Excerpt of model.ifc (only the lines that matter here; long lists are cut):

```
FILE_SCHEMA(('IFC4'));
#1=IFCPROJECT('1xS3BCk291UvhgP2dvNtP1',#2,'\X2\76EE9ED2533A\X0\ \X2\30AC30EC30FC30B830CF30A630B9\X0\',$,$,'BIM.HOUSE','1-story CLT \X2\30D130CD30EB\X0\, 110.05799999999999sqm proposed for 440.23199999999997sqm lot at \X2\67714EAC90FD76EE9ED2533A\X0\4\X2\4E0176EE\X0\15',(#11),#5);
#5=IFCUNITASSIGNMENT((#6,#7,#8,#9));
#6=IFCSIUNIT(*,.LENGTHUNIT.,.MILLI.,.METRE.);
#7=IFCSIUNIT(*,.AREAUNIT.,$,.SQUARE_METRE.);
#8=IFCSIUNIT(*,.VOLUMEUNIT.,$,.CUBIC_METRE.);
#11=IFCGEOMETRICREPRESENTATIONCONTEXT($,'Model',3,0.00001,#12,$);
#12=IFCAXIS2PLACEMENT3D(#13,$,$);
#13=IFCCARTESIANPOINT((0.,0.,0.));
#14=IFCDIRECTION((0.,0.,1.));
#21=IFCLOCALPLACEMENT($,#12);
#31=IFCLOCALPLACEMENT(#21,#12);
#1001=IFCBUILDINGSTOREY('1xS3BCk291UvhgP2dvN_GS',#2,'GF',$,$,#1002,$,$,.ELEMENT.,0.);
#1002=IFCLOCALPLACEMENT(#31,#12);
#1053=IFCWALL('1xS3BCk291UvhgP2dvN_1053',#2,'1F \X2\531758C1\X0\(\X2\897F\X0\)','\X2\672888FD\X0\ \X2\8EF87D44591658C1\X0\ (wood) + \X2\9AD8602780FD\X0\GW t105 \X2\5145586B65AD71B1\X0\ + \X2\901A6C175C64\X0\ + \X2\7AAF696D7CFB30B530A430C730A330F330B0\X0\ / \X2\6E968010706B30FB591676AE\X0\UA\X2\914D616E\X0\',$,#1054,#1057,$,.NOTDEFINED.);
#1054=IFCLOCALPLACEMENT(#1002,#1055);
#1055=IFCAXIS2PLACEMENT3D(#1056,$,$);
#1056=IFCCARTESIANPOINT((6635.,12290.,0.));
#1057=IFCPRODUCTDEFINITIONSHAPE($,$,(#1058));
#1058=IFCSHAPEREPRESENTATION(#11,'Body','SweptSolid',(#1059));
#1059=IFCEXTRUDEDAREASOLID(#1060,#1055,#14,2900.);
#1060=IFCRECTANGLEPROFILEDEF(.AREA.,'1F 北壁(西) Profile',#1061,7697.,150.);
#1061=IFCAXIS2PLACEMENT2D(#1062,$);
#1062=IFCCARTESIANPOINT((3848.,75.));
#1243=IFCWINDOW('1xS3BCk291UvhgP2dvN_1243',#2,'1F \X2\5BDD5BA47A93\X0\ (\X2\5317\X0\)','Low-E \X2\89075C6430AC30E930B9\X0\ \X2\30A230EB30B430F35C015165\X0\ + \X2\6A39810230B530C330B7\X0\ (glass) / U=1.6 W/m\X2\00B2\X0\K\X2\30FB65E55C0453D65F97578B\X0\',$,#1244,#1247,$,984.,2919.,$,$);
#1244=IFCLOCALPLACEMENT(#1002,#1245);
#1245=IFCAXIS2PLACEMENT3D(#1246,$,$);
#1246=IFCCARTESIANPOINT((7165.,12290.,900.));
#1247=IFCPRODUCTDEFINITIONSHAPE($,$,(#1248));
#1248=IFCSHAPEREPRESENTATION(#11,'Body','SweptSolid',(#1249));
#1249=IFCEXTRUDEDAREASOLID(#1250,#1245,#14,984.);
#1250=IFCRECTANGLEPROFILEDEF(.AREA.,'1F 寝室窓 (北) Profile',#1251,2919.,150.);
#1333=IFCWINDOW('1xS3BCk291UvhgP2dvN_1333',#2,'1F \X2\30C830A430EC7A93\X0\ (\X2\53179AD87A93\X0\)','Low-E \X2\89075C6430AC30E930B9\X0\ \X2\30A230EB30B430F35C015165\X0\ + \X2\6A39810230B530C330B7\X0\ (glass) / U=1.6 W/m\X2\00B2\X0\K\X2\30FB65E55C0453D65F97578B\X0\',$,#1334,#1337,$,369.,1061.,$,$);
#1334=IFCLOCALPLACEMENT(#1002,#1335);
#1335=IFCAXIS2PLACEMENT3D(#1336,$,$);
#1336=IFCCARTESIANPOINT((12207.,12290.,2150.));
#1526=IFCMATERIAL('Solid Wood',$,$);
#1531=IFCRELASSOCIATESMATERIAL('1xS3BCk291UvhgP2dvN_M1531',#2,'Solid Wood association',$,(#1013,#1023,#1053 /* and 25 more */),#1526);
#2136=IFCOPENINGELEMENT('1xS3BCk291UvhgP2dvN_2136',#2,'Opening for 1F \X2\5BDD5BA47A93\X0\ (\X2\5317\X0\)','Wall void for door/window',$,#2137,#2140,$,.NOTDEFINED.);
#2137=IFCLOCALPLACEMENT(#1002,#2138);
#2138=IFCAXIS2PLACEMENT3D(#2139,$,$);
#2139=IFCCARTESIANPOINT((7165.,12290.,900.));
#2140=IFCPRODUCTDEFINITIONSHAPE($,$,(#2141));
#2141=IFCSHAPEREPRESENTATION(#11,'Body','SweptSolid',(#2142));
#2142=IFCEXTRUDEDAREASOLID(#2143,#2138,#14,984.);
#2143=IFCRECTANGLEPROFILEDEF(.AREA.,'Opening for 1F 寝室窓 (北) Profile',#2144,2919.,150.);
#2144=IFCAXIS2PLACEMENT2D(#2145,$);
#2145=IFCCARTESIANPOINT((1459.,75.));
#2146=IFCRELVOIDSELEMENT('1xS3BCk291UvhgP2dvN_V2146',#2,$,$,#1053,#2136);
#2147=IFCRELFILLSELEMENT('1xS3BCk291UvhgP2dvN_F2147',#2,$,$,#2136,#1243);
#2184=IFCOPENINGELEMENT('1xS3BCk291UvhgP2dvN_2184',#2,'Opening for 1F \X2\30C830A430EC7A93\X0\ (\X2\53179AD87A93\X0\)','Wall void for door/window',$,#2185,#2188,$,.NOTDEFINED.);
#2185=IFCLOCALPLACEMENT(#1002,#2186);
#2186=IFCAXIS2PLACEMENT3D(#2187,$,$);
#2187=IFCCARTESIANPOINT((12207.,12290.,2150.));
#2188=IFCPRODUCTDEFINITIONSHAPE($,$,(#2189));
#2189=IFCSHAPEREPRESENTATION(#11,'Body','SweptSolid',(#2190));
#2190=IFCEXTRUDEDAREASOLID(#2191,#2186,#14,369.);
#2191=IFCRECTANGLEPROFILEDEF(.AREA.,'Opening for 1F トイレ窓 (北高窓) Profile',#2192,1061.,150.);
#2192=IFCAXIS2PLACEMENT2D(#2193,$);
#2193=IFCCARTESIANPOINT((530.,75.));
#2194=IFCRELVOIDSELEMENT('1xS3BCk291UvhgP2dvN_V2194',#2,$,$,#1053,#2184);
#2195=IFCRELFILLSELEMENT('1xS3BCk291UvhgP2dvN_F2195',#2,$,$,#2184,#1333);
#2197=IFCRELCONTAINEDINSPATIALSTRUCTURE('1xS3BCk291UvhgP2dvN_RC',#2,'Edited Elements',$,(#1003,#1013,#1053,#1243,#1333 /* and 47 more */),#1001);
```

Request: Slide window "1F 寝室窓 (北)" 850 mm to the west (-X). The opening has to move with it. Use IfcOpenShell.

```python
import ifcopenshell
import ifcopenshell.api.geometry
import ifcopenshell.util.placement
import ifcopenshell.util.unit

model = ifcopenshell.open("model.ifc")
unit_scale = ifcopenshell.util.unit.calculate_unit_scale(model)

window = model.by_guid("1xS3BCk291UvhgP2dvN_1243")
opening = window.FillsVoids[0].RelatingOpeningElement
wall = opening.VoidsElements[0].RelatingBuildingElement

wall_matrix = ifcopenshell.util.placement.get_local_placement(wall.ObjectPlacement)
shift = wall_matrix[:3, 0] * -0.85 / unit_scale
before = ifcopenshell.util.placement.get_local_placement(window.ObjectPlacement)[:3, 3].copy()

# The window is not placed relative to its opening, so move both.
for product in (opening, window):
    matrix = ifcopenshell.util.placement.get_local_placement(product.ObjectPlacement)
    matrix[:3, 3] += shift
    ifcopenshell.api.geometry.edit_object_placement(model, product=product, matrix=matrix, is_si=False)

after = ifcopenshell.util.placement.get_local_placement(window.ObjectPlacement)[:3, 3]
print("window moved by", (after - before).round(3) + 0.0)

model.write("model_v2.ifc")
```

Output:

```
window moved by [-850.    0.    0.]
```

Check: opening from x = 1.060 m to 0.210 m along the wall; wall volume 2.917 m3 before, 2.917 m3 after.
